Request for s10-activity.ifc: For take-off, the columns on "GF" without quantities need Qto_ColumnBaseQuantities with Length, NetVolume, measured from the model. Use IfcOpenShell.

First a look at what the model holds.

```python
import ifcopenshell
import ifcopenshell.util.element
import ifcopenshell.util.unit

model = ifcopenshell.open("s10-activity.ifc")
print(model.schema)
for unit_type in ("LENGTHUNIT", "AREAUNIT", "VOLUMEUNIT"):
    print(unit_type, ifcopenshell.util.unit.calculate_unit_scale(model, unit_type))
storey = next(s for s in model.by_type("IfcBuildingStorey") if s.Name == "GF")
columns = [e for e in ifcopenshell.util.element.get_decomposition(storey) if e.is_a("IfcColumn")]
for e in sorted(columns, key=lambda e: e.id()):
    print(e.id(), e.is_a(), e.Name, list(ifcopenshell.util.element.get_psets(e, qtos_only=True)), sep=" | ")
```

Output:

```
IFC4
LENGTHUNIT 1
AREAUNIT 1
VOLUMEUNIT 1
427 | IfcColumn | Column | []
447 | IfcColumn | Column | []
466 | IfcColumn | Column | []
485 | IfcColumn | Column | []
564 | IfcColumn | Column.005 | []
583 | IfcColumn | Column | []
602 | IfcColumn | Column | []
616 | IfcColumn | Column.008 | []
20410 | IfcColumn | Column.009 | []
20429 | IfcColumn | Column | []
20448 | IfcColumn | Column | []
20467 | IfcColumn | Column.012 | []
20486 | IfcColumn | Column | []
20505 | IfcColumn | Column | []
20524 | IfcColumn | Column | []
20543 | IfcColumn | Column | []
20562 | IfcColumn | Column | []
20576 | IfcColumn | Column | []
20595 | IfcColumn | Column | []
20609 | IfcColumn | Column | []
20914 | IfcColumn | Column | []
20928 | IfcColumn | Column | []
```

```python
import ifcopenshell
import ifcopenshell.api.pset
import ifcopenshell.geom
import ifcopenshell.util.element
import ifcopenshell.util.shape
import ifcopenshell.util.unit

model = ifcopenshell.open("s10-activity.ifc")
unit_scale = ifcopenshell.util.unit.calculate_unit_scale(model)
volume_scale = ifcopenshell.util.unit.calculate_unit_scale(model, "VOLUMEUNIT")
settings = ifcopenshell.geom.settings()

storey = next(s for s in model.by_type("IfcBuildingStorey") if s.Name == "GF")
columns = [e for e in ifcopenshell.util.element.get_decomposition(storey) if e.is_a("IfcColumn")]

for e in sorted(columns, key=lambda e: e.id()):
    if ifcopenshell.util.element.get_psets(e, qtos_only=True, should_inherit=False):
        continue
    # Geometry comes back in metres, in the element's own axes.
    shape = ifcopenshell.geom.create_shape(settings, e)
    values = {
        "Length": ifcopenshell.util.shape.get_z(shape.geometry) / unit_scale,
        "NetVolume": ifcopenshell.util.shape.get_volume(shape.geometry) / volume_scale,
    }
    qto = ifcopenshell.api.pset.add_qto(model, product=e, name="Qto_ColumnBaseQuantities")
    ifcopenshell.api.pset.edit_qto(model, qto=qto, properties=values)
    print(e.id(), {k: round(v, 3) for k, v in values.items()})

model.write("s10-activity_v2.ifc")
```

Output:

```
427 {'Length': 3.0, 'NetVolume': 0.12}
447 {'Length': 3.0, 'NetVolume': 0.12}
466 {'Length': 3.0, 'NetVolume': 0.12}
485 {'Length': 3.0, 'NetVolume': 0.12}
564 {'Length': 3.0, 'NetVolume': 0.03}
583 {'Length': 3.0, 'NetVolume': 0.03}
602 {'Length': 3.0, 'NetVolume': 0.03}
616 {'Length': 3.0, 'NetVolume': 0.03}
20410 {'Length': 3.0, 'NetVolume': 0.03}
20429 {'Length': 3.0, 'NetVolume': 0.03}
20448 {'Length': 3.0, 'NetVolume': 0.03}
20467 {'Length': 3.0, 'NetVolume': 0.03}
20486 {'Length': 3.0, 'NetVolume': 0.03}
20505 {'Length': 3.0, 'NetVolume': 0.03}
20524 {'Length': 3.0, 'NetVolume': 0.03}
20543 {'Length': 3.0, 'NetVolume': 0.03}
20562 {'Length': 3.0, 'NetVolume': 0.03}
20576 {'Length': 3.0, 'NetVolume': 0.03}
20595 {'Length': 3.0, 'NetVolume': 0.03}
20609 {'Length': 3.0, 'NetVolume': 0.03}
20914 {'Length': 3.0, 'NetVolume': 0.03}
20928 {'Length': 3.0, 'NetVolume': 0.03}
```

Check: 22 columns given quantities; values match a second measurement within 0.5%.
